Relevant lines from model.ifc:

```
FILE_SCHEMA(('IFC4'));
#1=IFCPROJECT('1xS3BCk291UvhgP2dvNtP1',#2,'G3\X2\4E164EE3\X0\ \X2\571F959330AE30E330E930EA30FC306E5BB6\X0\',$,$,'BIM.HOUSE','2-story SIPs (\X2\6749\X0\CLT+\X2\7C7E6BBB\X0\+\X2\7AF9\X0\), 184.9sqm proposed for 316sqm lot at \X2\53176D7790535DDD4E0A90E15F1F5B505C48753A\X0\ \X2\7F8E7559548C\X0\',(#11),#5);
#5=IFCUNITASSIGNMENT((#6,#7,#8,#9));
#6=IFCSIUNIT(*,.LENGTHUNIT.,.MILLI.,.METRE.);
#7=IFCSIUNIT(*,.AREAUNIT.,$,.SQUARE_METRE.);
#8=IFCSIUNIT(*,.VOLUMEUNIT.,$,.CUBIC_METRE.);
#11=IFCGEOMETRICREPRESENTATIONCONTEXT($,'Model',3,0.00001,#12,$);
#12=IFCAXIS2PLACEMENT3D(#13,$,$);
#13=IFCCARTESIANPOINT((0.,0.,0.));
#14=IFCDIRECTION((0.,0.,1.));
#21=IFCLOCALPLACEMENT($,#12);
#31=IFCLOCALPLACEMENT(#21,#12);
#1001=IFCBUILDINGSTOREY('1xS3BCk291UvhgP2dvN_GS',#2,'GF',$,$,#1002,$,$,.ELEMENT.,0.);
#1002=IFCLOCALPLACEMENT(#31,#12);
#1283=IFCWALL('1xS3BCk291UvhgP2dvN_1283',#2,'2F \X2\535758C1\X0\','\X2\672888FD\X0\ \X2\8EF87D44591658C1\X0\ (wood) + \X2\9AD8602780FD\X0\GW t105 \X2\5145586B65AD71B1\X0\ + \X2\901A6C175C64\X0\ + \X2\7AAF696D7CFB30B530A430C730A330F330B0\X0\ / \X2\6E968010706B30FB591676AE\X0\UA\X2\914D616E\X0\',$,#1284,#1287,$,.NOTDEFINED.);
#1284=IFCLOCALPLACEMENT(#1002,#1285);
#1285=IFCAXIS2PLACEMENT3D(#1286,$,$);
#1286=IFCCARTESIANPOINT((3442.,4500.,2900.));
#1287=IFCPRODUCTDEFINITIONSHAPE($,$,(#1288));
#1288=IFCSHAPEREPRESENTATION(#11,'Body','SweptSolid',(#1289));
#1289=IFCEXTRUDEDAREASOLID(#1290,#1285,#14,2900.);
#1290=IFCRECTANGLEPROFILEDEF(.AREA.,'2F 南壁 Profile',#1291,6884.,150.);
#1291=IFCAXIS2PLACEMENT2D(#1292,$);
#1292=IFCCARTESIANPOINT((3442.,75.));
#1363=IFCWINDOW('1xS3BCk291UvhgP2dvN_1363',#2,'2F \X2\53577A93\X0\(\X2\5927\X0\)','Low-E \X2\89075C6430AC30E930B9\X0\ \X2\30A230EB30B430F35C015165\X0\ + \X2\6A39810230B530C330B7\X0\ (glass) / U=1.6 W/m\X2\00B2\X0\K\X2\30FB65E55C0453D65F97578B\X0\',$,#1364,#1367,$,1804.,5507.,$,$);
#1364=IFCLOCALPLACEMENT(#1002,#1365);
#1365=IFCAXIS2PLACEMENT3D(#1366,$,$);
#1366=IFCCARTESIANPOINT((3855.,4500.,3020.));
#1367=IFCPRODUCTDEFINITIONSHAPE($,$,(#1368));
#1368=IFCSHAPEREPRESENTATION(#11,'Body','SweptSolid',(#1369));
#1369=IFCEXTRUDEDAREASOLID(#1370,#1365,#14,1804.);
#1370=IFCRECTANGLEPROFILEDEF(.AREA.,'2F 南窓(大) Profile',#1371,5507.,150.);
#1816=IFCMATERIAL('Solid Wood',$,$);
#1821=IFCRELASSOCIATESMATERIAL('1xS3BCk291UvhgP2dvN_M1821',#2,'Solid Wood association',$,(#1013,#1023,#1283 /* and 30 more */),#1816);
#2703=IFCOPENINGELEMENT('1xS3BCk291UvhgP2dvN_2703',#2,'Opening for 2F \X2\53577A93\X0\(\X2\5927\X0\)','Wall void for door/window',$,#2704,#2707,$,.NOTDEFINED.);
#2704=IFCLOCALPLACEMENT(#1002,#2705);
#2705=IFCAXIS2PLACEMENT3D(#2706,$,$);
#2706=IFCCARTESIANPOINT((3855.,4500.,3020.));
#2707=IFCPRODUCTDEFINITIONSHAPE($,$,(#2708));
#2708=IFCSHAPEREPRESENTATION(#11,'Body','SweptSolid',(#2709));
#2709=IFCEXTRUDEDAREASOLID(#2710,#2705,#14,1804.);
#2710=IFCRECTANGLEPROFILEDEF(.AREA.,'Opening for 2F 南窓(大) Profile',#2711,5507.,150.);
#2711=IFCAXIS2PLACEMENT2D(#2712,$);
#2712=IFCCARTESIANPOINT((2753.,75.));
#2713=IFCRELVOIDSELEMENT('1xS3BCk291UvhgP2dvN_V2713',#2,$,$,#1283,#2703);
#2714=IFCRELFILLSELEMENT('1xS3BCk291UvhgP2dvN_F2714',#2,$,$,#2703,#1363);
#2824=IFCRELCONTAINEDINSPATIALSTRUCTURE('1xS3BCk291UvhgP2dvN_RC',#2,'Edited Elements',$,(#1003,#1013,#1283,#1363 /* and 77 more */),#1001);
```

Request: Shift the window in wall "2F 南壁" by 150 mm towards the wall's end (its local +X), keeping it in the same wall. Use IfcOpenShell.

```python
import ifcopenshell
import ifcopenshell.api.geometry
import ifcopenshell.util.placement
import ifcopenshell.util.unit

model = ifcopenshell.open("model.ifc")
unit_scale = ifcopenshell.util.unit.calculate_unit_scale(model)

window = model.by_guid("1xS3BCk291UvhgP2dvN_1363")
opening = window.FillsVoids[0].RelatingOpeningElement
wall = opening.VoidsElements[0].RelatingBuildingElement

wall_matrix = ifcopenshell.util.placement.get_local_placement(wall.ObjectPlacement)
shift = wall_matrix[:3, 0] * 0.15 / unit_scale
before = ifcopenshell.util.placement.get_local_placement(window.ObjectPlacement)[:3, 3].copy()

# The window is not placed relative to its opening, so move both.
for product in (opening, window):
    matrix = ifcopenshell.util.placement.get_local_placement(product.ObjectPlacement)
    matrix[:3, 3] += shift
    ifcopenshell.api.geometry.edit_object_placement(model, product=product, matrix=matrix, is_si=False)

after = ifcopenshell.util.placement.get_local_placement(window.ObjectPlacement)[:3, 3]
print("window moved by", (after - before).round(3) + 0.0)

model.write("model_rev.ifc")
```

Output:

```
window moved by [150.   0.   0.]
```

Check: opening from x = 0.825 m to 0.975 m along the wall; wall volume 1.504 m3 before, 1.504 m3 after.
